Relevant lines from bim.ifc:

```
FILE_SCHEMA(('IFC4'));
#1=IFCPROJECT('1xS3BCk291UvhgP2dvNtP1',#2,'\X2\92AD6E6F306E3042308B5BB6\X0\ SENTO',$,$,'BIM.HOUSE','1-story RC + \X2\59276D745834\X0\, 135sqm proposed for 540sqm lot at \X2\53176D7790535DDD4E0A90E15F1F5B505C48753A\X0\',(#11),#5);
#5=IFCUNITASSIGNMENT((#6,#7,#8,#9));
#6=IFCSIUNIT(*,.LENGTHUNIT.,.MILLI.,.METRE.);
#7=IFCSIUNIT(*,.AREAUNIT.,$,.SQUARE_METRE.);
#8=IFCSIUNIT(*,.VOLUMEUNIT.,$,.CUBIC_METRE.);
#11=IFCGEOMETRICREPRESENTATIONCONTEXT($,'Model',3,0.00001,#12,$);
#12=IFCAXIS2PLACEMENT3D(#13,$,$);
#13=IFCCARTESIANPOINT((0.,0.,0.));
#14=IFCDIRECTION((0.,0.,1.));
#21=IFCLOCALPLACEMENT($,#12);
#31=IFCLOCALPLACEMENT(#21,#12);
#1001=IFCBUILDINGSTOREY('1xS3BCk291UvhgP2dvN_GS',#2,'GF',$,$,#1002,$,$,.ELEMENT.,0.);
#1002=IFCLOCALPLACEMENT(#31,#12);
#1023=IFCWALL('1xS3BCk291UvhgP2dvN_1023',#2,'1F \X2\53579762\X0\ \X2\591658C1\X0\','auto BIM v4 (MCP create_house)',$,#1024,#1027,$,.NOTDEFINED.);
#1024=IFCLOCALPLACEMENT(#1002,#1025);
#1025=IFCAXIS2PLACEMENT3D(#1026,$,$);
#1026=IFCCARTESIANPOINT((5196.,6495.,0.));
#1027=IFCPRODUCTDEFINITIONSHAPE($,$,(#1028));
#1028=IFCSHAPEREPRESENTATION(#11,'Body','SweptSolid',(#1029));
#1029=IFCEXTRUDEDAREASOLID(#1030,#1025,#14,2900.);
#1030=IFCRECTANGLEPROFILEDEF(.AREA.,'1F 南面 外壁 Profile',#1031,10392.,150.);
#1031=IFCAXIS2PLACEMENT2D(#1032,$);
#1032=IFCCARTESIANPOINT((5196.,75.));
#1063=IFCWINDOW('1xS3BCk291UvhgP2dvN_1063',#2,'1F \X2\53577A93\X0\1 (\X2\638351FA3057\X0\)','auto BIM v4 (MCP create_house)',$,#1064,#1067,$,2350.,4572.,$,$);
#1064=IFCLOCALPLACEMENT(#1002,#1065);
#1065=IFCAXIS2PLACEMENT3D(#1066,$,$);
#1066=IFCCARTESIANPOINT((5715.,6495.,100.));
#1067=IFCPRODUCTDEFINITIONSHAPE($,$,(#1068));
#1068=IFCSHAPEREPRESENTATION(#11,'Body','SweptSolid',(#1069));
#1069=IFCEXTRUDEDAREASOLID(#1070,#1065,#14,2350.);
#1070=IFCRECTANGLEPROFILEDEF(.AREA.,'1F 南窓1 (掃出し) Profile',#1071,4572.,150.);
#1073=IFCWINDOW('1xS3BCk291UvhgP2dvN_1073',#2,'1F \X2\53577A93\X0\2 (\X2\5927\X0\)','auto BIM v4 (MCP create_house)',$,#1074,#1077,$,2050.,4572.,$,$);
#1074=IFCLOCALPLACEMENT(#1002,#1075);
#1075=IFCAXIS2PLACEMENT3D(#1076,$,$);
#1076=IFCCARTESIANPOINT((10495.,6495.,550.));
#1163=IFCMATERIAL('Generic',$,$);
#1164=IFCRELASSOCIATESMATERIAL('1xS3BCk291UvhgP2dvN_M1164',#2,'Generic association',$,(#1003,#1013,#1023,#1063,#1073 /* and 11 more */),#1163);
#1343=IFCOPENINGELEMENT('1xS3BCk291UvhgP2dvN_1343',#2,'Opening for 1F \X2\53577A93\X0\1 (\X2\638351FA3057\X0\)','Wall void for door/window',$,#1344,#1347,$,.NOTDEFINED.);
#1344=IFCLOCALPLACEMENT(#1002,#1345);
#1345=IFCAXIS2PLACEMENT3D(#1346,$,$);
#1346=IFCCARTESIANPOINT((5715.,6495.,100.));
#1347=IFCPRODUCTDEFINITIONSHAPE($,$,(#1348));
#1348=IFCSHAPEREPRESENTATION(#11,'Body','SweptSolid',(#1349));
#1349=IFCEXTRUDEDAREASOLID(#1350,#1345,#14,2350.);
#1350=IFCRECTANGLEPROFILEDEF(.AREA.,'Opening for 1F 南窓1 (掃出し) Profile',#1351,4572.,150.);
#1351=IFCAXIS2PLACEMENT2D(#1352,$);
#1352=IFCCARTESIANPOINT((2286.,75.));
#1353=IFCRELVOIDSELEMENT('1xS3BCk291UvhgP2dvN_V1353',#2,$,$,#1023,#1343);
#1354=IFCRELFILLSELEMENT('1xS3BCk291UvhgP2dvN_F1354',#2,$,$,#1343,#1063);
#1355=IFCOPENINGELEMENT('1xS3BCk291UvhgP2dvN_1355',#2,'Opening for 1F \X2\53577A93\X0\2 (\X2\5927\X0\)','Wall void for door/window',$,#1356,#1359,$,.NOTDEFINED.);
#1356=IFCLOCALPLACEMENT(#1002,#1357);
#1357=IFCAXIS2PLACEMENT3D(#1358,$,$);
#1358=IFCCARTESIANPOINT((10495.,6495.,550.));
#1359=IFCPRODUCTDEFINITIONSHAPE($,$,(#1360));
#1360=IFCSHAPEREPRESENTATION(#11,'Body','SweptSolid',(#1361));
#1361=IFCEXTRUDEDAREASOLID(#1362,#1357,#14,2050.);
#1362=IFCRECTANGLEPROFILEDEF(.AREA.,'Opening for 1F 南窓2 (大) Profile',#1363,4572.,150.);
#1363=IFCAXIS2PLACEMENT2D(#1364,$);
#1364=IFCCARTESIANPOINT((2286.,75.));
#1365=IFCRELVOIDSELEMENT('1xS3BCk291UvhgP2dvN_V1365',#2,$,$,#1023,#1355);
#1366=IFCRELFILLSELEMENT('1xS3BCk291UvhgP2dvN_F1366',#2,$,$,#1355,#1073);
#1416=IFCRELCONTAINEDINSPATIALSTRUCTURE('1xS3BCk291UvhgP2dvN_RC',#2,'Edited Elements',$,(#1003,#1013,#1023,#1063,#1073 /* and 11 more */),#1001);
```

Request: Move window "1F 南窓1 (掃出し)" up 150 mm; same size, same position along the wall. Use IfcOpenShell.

```python
import numpy as np
import ifcopenshell
import ifcopenshell.api.geometry
import ifcopenshell.util.placement
import ifcopenshell.util.unit

model = ifcopenshell.open("bim.ifc")
unit_scale = ifcopenshell.util.unit.calculate_unit_scale(model)

window = model.by_guid("1xS3BCk291UvhgP2dvN_1063")
opening = window.FillsVoids[0].RelatingOpeningElement
dz = 150.0

shift = np.array([0.0, 0.0, dz])
# The window is not placed relative to its opening, so move both.
for product in (opening, window):
    matrix = ifcopenshell.util.placement.get_local_placement(product.ObjectPlacement)
    matrix[:3, 3] += shift
    ifcopenshell.api.geometry.edit_object_placement(model, product=product, matrix=matrix, is_si=False)

print(f"moved by {dz * unit_scale:+.3f} m")

model.write("bim_updated.ifc")
```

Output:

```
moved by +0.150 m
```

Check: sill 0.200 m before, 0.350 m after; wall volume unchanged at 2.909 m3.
